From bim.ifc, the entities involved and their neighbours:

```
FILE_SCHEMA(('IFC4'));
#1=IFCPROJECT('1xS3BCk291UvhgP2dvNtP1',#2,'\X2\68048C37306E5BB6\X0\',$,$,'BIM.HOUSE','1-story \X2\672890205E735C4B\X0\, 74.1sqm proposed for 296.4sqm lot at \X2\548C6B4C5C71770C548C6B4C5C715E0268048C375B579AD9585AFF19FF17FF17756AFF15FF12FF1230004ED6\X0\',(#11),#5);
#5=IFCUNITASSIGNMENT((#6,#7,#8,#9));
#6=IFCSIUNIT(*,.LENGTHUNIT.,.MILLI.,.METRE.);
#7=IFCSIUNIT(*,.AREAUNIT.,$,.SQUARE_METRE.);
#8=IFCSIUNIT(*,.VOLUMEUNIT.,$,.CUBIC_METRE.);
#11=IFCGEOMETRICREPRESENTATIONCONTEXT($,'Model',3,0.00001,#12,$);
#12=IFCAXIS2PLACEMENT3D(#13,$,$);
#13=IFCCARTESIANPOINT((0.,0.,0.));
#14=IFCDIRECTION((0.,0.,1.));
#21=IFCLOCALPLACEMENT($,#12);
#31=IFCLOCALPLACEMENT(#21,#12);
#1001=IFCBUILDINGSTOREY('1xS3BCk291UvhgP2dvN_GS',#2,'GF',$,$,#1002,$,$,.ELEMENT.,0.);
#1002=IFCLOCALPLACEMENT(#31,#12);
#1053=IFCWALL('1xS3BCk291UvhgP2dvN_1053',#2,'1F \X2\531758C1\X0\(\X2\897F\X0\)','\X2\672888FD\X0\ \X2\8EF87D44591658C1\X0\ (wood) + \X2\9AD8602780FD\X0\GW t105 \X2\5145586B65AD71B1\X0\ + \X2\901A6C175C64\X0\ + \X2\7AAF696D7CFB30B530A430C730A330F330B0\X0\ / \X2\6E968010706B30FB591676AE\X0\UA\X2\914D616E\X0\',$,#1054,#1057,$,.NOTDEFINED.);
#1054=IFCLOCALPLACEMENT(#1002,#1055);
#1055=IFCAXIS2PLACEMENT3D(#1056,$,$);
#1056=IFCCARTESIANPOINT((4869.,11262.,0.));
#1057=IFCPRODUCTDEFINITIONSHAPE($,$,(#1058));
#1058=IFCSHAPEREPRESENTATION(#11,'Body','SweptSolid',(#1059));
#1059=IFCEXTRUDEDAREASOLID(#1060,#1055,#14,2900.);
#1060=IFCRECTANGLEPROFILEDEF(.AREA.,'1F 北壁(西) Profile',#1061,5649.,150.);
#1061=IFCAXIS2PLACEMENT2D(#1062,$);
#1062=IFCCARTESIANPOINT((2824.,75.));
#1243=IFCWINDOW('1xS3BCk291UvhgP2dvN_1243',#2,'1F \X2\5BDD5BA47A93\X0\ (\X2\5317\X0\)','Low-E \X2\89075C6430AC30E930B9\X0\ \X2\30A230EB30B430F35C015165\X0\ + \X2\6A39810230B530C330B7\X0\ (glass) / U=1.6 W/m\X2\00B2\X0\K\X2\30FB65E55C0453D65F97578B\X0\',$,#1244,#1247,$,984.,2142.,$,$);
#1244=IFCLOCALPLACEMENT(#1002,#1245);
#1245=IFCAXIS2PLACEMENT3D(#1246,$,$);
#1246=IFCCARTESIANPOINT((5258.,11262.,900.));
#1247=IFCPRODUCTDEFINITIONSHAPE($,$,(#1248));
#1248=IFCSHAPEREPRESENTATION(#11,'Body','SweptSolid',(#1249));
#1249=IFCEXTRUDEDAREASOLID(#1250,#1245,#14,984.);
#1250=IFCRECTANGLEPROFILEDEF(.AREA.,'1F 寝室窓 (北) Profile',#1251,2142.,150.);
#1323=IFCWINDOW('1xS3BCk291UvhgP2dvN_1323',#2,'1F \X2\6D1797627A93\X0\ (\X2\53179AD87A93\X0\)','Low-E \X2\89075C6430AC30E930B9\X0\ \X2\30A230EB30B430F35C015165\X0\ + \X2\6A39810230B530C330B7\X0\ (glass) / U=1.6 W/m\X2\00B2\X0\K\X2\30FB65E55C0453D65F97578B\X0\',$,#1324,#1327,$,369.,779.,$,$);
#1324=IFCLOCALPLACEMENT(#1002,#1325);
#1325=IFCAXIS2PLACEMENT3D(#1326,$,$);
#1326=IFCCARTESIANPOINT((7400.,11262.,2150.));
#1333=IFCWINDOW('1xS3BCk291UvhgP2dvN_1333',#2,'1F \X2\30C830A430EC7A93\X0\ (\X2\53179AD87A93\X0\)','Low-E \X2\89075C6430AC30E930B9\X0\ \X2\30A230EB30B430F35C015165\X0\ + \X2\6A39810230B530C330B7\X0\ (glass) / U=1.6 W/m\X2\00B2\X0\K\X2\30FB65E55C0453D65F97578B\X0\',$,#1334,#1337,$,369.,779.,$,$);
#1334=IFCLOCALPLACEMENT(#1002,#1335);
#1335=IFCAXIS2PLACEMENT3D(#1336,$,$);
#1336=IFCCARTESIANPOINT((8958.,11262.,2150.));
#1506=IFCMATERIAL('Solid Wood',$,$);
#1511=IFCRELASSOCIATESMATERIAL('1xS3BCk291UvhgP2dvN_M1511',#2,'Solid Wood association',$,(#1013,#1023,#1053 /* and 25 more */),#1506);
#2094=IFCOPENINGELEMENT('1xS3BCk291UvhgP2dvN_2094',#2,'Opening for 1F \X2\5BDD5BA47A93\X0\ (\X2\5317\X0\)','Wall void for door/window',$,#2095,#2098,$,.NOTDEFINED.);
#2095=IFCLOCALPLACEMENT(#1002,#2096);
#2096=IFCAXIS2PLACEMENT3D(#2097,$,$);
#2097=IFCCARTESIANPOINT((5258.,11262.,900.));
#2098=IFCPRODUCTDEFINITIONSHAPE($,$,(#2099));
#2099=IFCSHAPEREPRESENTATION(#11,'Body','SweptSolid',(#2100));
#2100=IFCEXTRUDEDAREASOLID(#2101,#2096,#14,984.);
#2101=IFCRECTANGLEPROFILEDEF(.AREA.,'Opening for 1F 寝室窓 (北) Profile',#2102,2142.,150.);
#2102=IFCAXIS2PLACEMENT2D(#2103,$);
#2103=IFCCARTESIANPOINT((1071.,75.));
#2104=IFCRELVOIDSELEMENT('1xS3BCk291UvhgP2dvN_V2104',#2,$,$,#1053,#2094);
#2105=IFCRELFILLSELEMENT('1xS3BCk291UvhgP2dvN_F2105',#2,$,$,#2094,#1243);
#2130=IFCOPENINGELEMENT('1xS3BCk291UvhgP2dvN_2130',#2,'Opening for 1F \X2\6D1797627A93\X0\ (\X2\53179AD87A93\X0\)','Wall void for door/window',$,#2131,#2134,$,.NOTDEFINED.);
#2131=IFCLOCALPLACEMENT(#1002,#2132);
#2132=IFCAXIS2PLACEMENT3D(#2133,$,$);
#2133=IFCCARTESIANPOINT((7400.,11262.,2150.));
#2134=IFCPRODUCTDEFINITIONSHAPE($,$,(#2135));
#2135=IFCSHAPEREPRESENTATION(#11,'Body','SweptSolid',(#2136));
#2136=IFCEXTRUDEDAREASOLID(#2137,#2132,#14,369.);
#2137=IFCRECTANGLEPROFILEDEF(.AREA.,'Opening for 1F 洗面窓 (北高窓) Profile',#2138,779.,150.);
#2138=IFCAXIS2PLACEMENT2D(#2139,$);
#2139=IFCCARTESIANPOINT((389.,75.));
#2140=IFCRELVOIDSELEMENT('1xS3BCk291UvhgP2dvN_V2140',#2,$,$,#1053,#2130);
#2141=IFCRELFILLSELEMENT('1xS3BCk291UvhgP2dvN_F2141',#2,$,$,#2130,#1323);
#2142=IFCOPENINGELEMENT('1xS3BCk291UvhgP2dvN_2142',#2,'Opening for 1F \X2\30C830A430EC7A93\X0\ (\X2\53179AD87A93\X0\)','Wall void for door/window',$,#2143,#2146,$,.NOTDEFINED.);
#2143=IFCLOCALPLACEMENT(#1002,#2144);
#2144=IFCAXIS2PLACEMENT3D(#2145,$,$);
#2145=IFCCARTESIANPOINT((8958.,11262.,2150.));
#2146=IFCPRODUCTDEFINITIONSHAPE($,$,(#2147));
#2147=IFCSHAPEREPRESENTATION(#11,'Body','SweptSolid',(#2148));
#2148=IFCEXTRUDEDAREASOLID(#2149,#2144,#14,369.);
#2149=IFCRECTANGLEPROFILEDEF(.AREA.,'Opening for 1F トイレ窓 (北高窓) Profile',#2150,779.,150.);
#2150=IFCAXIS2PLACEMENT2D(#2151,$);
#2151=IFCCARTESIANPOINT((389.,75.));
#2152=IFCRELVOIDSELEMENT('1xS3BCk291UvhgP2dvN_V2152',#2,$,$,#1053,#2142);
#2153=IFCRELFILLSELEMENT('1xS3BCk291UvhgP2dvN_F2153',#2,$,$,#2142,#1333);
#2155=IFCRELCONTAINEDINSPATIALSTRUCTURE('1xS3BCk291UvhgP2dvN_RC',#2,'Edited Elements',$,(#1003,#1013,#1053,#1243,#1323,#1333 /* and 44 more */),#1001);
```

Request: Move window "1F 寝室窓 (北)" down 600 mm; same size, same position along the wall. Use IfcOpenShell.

```python
import numpy as np
import ifcopenshell
import ifcopenshell.api.geometry
import ifcopenshell.util.placement
import ifcopenshell.util.unit

model = ifcopenshell.open("bim.ifc")
unit_scale = ifcopenshell.util.unit.calculate_unit_scale(model)

window = model.by_guid("1xS3BCk291UvhgP2dvN_1243")
opening = window.FillsVoids[0].RelatingOpeningElement
dz = -0.6 / unit_scale

shift = np.array([0.0, 0.0, dz])
# The window is not placed relative to its opening, so move both.
for product in (opening, window):
    matrix = ifcopenshell.util.placement.get_local_placement(product.ObjectPlacement)
    matrix[:3, 3] += shift
    ifcopenshell.api.geometry.edit_object_placement(model, product=product, matrix=matrix, is_si=False)

print(f"moved by {dz * unit_scale:+.3f} m")

model.write("bim_edited.ifc")
```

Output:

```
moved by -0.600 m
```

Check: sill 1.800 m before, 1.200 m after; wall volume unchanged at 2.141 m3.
